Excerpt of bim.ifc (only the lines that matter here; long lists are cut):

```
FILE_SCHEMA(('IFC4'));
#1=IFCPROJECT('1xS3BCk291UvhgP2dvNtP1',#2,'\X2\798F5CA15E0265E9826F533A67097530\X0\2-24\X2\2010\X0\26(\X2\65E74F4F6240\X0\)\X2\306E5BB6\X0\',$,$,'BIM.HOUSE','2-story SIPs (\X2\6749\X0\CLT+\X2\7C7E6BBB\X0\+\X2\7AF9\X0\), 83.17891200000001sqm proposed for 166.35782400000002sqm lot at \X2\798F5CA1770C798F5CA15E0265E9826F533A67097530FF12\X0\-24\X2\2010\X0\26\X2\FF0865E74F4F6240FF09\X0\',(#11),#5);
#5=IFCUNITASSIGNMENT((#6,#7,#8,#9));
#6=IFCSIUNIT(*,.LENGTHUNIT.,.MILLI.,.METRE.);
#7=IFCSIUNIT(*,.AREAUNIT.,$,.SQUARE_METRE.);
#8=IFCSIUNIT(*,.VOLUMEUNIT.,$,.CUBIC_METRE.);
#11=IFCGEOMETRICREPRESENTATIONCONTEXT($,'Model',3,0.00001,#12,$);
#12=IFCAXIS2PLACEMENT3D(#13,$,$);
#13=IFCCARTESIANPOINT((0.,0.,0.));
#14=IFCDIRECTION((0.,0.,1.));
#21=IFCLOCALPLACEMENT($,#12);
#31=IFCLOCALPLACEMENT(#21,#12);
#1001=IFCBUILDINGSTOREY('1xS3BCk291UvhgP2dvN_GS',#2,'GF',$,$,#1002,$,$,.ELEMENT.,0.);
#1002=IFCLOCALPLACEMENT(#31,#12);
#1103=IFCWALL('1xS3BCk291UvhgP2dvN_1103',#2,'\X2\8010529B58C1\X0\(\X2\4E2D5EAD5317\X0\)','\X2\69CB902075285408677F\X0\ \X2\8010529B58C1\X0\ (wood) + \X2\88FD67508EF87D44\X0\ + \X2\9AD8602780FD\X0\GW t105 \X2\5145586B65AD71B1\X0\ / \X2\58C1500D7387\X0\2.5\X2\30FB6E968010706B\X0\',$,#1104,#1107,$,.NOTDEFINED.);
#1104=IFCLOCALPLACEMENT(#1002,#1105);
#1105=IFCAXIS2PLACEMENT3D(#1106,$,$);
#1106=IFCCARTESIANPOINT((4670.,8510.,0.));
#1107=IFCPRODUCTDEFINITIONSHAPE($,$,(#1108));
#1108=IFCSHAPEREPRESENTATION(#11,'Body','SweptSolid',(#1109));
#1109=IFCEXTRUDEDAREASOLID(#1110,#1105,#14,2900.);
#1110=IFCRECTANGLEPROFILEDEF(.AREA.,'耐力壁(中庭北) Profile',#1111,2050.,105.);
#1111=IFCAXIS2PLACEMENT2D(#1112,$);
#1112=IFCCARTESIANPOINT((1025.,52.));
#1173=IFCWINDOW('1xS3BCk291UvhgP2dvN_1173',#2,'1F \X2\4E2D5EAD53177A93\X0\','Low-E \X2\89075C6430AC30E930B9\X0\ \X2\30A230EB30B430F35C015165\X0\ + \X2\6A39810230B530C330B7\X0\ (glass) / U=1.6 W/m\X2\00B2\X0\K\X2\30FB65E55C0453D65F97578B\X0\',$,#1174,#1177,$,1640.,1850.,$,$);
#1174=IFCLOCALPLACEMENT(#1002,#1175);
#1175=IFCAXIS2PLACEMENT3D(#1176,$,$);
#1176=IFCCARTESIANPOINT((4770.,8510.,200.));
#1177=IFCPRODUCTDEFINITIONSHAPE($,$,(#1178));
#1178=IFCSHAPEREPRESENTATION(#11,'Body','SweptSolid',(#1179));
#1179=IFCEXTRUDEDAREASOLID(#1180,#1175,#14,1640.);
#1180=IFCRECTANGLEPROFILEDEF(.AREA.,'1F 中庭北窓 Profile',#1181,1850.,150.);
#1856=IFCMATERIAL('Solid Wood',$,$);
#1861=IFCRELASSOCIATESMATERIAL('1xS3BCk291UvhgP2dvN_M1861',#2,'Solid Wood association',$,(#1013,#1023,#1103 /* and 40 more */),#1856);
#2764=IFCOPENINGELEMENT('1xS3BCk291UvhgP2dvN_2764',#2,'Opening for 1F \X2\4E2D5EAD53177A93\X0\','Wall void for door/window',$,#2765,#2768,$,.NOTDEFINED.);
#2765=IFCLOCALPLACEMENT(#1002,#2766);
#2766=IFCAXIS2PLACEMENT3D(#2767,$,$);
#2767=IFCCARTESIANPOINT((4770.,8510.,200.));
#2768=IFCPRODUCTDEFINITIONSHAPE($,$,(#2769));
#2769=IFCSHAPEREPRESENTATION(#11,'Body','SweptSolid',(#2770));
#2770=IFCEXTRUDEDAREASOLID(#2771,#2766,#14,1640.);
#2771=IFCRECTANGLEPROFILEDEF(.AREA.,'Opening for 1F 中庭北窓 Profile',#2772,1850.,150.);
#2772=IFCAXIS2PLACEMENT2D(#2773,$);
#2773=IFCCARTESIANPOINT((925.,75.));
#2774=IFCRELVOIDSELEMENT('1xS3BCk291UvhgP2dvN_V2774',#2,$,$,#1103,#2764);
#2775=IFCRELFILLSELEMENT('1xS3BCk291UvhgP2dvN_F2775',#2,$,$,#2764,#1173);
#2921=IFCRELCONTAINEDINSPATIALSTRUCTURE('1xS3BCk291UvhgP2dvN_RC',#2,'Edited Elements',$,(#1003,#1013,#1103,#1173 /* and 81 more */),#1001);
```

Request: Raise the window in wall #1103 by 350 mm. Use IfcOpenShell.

```python
import numpy as np
import ifcopenshell
import ifcopenshell.api.geometry
import ifcopenshell.util.placement
import ifcopenshell.util.unit

model = ifcopenshell.open("bim.ifc")
unit_scale = ifcopenshell.util.unit.calculate_unit_scale(model)

window = model.by_guid("1xS3BCk291UvhgP2dvN_1173")
opening = window.FillsVoids[0].RelatingOpeningElement
dz = 0.35 / unit_scale

shift = np.array([0.0, 0.0, dz])
# The window is not placed relative to its opening, so move both.
for product in (opening, window):
    matrix = ifcopenshell.util.placement.get_local_placement(product.ObjectPlacement)
    matrix[:3, 3] += shift
    ifcopenshell.api.geometry.edit_object_placement(model, product=product, matrix=matrix, is_si=False)

print(f"moved by {dz * unit_scale:+.3f} m")

model.write("bim_v2.ifc")
```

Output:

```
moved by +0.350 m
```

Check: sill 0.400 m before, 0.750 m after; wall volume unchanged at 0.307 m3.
